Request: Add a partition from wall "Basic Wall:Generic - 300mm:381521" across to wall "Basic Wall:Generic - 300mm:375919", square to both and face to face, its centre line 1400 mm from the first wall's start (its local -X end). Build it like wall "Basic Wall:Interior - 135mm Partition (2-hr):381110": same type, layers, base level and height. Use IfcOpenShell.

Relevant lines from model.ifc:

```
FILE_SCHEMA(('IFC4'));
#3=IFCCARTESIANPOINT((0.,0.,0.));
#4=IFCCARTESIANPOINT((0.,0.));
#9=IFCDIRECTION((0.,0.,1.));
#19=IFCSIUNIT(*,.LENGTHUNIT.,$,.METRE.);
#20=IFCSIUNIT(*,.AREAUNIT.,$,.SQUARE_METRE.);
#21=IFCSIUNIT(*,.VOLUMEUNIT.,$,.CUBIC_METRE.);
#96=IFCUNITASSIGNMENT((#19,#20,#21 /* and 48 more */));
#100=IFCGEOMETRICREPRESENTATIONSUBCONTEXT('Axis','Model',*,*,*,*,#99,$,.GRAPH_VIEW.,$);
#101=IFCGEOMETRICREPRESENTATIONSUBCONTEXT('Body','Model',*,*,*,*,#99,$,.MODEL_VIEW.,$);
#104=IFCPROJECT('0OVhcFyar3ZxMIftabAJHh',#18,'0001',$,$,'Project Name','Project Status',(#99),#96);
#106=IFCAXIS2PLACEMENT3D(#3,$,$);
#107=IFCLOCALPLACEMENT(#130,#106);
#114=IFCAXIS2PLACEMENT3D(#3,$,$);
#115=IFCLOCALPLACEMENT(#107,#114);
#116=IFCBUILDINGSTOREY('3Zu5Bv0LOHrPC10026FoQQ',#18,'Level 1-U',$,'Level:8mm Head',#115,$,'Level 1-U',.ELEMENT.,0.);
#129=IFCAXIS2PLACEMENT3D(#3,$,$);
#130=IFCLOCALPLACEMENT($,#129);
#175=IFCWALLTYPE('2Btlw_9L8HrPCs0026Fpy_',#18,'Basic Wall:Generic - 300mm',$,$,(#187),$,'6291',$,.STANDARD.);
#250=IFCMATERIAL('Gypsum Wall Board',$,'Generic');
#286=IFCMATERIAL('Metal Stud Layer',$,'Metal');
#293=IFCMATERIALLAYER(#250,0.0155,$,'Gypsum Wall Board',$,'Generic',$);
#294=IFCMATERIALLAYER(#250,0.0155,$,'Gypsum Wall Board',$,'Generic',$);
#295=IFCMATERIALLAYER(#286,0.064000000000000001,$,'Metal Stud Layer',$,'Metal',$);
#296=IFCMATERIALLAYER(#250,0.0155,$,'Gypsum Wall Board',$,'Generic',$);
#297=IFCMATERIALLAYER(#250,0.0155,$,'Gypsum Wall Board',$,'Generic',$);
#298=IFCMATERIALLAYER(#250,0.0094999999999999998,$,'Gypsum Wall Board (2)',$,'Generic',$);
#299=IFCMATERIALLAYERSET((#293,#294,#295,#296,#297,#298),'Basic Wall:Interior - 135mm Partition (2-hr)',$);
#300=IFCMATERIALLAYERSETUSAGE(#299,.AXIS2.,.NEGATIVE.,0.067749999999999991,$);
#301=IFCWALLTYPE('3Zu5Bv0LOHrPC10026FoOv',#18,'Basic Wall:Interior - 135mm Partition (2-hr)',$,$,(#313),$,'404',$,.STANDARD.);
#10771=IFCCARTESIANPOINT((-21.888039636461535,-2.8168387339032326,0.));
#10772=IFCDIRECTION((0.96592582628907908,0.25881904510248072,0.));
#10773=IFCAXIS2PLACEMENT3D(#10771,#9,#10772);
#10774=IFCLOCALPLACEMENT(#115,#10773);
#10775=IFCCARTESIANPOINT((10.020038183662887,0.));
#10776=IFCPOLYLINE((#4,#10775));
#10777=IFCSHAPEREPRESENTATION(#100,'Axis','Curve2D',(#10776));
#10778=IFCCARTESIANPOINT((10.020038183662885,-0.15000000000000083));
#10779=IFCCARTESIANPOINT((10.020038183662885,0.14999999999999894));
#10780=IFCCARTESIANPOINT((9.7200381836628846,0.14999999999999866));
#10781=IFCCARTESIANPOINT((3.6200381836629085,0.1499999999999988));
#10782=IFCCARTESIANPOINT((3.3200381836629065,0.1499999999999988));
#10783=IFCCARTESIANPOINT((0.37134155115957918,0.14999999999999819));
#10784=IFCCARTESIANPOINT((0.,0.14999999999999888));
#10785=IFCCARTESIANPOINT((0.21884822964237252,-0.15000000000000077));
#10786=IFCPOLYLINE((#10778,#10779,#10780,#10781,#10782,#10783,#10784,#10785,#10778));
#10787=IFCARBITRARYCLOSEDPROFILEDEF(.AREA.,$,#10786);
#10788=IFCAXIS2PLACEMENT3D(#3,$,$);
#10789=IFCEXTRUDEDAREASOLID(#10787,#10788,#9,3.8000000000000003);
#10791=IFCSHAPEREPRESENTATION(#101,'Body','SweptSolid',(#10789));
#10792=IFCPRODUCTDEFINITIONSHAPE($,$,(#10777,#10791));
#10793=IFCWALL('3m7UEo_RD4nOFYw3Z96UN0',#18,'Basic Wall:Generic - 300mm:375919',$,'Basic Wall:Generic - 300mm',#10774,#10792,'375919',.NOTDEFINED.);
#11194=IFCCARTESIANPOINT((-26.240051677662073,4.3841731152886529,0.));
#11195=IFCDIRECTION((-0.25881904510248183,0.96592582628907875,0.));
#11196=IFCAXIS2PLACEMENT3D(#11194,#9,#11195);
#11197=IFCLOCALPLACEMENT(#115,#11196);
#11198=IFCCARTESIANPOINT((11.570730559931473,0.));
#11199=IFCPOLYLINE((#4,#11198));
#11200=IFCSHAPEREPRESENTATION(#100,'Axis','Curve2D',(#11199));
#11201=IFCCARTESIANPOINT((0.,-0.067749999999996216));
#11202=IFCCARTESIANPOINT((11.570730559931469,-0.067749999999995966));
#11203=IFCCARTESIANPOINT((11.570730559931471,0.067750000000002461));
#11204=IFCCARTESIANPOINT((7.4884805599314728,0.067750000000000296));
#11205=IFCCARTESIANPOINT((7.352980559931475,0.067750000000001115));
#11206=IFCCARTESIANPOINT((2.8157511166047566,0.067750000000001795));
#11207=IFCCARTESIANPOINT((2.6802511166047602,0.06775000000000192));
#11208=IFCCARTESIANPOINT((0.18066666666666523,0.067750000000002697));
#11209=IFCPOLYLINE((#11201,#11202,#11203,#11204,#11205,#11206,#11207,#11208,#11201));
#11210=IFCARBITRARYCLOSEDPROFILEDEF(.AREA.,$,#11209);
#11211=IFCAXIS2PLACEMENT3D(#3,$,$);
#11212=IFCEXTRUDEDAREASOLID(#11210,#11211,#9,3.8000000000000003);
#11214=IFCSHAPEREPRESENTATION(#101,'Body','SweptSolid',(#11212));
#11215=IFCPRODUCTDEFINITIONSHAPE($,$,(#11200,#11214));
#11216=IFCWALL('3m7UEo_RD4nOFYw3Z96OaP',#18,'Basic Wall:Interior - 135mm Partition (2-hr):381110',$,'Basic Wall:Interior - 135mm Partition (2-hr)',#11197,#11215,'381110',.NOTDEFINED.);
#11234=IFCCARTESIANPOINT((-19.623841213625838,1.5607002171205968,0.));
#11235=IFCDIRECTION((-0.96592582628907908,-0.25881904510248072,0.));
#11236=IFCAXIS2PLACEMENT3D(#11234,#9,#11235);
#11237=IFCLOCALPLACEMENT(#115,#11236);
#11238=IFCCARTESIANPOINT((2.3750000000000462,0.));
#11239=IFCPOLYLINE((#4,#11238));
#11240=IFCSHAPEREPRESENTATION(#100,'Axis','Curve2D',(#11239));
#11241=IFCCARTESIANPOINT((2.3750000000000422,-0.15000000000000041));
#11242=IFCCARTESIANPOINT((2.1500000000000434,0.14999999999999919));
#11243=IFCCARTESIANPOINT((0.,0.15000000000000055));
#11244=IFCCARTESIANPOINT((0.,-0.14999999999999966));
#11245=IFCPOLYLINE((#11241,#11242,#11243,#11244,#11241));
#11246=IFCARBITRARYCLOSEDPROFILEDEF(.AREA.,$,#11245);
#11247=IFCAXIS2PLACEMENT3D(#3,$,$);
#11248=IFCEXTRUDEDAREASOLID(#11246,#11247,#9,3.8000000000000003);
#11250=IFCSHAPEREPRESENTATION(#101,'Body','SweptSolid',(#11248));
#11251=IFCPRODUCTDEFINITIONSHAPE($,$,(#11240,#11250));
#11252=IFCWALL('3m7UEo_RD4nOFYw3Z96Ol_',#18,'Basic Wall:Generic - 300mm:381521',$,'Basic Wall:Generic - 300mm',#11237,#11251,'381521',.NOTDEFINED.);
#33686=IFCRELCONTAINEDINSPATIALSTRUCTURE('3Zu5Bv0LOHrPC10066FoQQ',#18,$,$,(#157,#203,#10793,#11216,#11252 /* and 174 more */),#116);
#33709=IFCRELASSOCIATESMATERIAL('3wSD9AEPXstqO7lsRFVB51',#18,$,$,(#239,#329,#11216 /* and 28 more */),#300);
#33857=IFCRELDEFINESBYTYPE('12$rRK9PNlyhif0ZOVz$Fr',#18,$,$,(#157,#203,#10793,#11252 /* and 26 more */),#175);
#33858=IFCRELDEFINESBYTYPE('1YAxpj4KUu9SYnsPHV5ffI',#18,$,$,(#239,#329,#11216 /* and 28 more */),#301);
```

```python
import numpy as np
import ifcopenshell
import ifcopenshell.api.geometry
import ifcopenshell.api.material
import ifcopenshell.api.pset
import ifcopenshell.api.root
import ifcopenshell.api.spatial
import ifcopenshell.api.type
import ifcopenshell.geom
import ifcopenshell.util.element
import ifcopenshell.util.placement
import ifcopenshell.util.representation
import ifcopenshell.util.shape
import ifcopenshell.util.unit

model = ifcopenshell.open("model.ifc")
unit_scale = ifcopenshell.util.unit.calculate_unit_scale(model)
settings = ifcopenshell.geom.settings()
settings.set("use-world-coords", True)

start_wall = model.by_guid("3m7UEo_RD4nOFYw3Z96Ol_")
end_wall = model.by_guid("3m7UEo_RD4nOFYw3Z96UN0")
like = model.by_guid("3m7UEo_RD4nOFYw3Z96OaP")
matrix = ifcopenshell.util.placement.get_local_placement(start_wall.ObjectPlacement)
matrix[:3, 3] *= unit_scale


def extent(element):
    """Bounding box in the first wall's axes, in metres."""
    shape = ifcopenshell.geom.create_shape(settings, element)
    points = (ifcopenshell.util.shape.get_vertices(shape.geometry) - matrix[:3, 3]) @ matrix[:3, :3]
    return points.min(axis=0), points.max(axis=0)


y_start = extent(start_wall)[1][1]
y_end = extent(end_wall)[0][1]
like_min, like_max = extent(like)
length, height = float(abs(y_end - y_start)), float(like_max[2] - like_min[2])
layer_set = ifcopenshell.util.element.get_material(like, should_skip_usage=True)
thickness = sum(layer.LayerThickness for layer in layer_set.MaterialLayers) * unit_scale

wall = ifcopenshell.api.root.create_entity(model, ifc_class="IfcWall", name="New partition")
storey = ifcopenshell.util.element.get_container(like)
ifcopenshell.api.spatial.assign_container(model, products=[wall], relating_structure=storey)
ifcopenshell.api.type.assign_type(
    model, related_objects=[wall], relating_type=ifcopenshell.util.element.get_type(like), should_map_representations=False
)
rel = ifcopenshell.api.material.assign_material(
    model, products=[wall], type="IfcMaterialLayerSetUsage", material=layer_set
)
rel.RelatingMaterial.OffsetFromReferenceLine = -thickness / 2 / unit_scale
pset = ifcopenshell.api.pset.add_pset(model, product=wall, name="Pset_WallCommon")
ifcopenshell.api.pset.edit_pset(model, pset=pset, properties={"IsExternal": False, "LoadBearing": False})

# The axis runs down the middle of the wall.
axis = ifcopenshell.api.geometry.add_axis_representation(
    model, context=ifcopenshell.util.representation.get_context(model, "Model", "Axis"), axis=[(0.0, 0.0), (length, 0.0)]
)
body = ifcopenshell.api.geometry.add_wall_representation(
    model,
    context=ifcopenshell.util.representation.get_context(model, "Model", "Body", "MODEL_VIEW"),
    length=length,
    height=height,
    thickness=thickness,
    offset=-thickness / 2,
)
for representation in (axis, body):
    ifcopenshell.api.geometry.assign_representation(model, product=wall, representation=representation)

placement = matrix @ ifcopenshell.util.placement.rotation(90, "Z")
placement[:, 3] = matrix @ np.array([extent(start_wall)[0][0] + 1.4, y_start, like_min[2], 1.0])
ifcopenshell.api.geometry.edit_object_placement(model, product=wall, matrix=placement)

print(f"partition {length:.3f} m long, {height:.3f} m high, {thickness:.3f} m thick")

model.write("model_v2.ifc")
```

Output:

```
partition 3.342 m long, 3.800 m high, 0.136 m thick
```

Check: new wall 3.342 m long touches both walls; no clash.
